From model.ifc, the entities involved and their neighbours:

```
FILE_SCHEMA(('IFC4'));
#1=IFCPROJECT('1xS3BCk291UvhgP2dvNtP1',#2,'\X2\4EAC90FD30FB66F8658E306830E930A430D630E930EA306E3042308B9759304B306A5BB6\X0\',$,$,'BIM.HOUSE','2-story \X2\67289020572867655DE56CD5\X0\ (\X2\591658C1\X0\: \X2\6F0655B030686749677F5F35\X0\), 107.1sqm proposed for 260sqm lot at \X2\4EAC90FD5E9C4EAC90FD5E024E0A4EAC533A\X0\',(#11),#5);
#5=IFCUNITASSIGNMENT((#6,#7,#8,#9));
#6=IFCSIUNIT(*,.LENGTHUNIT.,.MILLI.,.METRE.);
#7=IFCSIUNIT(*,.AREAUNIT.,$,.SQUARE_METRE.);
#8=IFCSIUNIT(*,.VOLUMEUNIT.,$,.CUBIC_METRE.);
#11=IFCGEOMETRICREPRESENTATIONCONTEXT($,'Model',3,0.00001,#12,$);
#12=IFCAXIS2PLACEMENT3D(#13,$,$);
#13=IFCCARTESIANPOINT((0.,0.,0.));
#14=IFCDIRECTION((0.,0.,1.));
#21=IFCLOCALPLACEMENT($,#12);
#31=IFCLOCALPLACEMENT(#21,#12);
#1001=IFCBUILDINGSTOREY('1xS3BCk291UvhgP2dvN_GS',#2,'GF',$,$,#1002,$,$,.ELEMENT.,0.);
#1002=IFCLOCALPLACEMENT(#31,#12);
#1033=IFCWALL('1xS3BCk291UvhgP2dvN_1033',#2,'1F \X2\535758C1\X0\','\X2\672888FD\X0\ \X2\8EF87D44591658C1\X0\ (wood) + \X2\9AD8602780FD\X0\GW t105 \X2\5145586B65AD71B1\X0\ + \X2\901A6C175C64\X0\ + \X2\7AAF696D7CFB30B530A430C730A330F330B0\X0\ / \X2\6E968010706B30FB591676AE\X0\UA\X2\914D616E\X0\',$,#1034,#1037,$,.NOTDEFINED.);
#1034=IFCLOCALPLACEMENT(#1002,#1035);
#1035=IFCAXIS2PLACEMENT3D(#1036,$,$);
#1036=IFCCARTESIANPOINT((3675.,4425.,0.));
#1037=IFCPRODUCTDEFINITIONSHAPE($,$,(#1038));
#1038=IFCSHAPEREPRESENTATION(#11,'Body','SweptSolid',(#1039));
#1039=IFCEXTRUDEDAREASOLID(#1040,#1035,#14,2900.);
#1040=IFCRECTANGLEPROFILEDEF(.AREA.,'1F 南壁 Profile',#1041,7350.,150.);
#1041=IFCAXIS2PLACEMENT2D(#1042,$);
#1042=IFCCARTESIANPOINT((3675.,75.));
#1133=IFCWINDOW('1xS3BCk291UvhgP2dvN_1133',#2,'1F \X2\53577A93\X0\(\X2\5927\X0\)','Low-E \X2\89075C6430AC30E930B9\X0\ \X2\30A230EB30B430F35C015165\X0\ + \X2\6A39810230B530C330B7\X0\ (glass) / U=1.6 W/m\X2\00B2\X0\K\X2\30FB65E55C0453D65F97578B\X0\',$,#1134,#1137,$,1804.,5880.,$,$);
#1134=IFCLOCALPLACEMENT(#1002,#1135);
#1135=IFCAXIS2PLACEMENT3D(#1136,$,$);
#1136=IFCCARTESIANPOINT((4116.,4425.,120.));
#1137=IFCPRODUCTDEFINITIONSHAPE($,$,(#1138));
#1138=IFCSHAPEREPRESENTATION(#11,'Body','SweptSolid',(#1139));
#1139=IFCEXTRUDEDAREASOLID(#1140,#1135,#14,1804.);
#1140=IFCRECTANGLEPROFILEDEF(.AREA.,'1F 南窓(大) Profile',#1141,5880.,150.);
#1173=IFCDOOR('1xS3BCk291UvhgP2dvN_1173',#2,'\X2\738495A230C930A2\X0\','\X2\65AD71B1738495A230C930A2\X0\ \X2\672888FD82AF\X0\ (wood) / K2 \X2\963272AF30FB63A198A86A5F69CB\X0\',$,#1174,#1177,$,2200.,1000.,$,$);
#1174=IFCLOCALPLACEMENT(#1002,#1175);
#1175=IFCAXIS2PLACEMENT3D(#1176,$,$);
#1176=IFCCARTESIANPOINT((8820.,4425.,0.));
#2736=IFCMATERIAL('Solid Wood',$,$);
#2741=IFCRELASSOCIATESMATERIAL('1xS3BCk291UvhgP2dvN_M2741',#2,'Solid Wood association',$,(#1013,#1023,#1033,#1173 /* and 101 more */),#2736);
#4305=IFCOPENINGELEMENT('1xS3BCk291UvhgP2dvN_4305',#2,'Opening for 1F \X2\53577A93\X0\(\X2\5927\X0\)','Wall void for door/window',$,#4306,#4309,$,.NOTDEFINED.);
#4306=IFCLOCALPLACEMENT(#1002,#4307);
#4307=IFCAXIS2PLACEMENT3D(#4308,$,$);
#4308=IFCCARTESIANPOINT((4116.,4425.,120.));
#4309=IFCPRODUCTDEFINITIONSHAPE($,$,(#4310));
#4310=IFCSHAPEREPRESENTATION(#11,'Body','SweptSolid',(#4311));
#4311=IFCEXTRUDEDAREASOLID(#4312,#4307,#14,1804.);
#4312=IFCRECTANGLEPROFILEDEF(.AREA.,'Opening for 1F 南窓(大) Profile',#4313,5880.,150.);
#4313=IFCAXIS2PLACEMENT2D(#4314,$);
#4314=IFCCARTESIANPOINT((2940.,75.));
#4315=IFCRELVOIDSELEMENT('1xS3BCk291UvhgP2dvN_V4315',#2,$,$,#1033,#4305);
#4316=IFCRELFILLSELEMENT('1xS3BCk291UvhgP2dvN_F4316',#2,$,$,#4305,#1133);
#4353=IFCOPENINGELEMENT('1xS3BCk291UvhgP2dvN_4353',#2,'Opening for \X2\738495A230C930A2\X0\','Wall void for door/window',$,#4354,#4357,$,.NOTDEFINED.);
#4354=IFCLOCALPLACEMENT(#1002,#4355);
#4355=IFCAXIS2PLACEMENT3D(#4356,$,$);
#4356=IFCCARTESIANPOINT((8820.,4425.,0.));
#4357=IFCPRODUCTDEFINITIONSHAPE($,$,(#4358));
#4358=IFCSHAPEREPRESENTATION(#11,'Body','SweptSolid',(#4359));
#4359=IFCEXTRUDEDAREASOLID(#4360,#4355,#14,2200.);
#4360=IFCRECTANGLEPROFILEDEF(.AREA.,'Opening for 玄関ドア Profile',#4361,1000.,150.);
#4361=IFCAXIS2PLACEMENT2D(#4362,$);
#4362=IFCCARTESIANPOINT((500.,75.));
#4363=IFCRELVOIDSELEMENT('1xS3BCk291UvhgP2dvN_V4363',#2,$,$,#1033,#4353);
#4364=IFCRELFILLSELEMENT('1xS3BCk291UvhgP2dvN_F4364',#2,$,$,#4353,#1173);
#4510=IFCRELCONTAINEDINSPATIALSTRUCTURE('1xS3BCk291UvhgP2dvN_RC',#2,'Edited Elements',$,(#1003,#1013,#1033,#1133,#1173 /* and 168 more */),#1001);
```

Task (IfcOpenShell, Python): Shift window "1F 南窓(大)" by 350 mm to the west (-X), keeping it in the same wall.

```python
import ifcopenshell
import ifcopenshell.api.geometry
import ifcopenshell.util.placement

model = ifcopenshell.open("model.ifc")

window = model.by_guid("1xS3BCk291UvhgP2dvN_1133")
opening = window.FillsVoids[0].RelatingOpeningElement
wall = opening.VoidsElements[0].RelatingBuildingElement

wall_matrix = ifcopenshell.util.placement.get_local_placement(wall.ObjectPlacement)
shift = wall_matrix[:3, 0] * -350.0
before = ifcopenshell.util.placement.get_local_placement(window.ObjectPlacement)[:3, 3].copy()

# The window is not placed relative to its opening, so move both.
for product in (opening, window):
    matrix = ifcopenshell.util.placement.get_local_placement(product.ObjectPlacement)
    matrix[:3, 3] += shift
    ifcopenshell.api.geometry.edit_object_placement(model, product=product, matrix=matrix, is_si=False)

after = ifcopenshell.util.placement.get_local_placement(window.ObjectPlacement)[:3, 3]
print("window moved by", (after - before).round(3) + 0.0)

model.write("model_v2.ifc")
```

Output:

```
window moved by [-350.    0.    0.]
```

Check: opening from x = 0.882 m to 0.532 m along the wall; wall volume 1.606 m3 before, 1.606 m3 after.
